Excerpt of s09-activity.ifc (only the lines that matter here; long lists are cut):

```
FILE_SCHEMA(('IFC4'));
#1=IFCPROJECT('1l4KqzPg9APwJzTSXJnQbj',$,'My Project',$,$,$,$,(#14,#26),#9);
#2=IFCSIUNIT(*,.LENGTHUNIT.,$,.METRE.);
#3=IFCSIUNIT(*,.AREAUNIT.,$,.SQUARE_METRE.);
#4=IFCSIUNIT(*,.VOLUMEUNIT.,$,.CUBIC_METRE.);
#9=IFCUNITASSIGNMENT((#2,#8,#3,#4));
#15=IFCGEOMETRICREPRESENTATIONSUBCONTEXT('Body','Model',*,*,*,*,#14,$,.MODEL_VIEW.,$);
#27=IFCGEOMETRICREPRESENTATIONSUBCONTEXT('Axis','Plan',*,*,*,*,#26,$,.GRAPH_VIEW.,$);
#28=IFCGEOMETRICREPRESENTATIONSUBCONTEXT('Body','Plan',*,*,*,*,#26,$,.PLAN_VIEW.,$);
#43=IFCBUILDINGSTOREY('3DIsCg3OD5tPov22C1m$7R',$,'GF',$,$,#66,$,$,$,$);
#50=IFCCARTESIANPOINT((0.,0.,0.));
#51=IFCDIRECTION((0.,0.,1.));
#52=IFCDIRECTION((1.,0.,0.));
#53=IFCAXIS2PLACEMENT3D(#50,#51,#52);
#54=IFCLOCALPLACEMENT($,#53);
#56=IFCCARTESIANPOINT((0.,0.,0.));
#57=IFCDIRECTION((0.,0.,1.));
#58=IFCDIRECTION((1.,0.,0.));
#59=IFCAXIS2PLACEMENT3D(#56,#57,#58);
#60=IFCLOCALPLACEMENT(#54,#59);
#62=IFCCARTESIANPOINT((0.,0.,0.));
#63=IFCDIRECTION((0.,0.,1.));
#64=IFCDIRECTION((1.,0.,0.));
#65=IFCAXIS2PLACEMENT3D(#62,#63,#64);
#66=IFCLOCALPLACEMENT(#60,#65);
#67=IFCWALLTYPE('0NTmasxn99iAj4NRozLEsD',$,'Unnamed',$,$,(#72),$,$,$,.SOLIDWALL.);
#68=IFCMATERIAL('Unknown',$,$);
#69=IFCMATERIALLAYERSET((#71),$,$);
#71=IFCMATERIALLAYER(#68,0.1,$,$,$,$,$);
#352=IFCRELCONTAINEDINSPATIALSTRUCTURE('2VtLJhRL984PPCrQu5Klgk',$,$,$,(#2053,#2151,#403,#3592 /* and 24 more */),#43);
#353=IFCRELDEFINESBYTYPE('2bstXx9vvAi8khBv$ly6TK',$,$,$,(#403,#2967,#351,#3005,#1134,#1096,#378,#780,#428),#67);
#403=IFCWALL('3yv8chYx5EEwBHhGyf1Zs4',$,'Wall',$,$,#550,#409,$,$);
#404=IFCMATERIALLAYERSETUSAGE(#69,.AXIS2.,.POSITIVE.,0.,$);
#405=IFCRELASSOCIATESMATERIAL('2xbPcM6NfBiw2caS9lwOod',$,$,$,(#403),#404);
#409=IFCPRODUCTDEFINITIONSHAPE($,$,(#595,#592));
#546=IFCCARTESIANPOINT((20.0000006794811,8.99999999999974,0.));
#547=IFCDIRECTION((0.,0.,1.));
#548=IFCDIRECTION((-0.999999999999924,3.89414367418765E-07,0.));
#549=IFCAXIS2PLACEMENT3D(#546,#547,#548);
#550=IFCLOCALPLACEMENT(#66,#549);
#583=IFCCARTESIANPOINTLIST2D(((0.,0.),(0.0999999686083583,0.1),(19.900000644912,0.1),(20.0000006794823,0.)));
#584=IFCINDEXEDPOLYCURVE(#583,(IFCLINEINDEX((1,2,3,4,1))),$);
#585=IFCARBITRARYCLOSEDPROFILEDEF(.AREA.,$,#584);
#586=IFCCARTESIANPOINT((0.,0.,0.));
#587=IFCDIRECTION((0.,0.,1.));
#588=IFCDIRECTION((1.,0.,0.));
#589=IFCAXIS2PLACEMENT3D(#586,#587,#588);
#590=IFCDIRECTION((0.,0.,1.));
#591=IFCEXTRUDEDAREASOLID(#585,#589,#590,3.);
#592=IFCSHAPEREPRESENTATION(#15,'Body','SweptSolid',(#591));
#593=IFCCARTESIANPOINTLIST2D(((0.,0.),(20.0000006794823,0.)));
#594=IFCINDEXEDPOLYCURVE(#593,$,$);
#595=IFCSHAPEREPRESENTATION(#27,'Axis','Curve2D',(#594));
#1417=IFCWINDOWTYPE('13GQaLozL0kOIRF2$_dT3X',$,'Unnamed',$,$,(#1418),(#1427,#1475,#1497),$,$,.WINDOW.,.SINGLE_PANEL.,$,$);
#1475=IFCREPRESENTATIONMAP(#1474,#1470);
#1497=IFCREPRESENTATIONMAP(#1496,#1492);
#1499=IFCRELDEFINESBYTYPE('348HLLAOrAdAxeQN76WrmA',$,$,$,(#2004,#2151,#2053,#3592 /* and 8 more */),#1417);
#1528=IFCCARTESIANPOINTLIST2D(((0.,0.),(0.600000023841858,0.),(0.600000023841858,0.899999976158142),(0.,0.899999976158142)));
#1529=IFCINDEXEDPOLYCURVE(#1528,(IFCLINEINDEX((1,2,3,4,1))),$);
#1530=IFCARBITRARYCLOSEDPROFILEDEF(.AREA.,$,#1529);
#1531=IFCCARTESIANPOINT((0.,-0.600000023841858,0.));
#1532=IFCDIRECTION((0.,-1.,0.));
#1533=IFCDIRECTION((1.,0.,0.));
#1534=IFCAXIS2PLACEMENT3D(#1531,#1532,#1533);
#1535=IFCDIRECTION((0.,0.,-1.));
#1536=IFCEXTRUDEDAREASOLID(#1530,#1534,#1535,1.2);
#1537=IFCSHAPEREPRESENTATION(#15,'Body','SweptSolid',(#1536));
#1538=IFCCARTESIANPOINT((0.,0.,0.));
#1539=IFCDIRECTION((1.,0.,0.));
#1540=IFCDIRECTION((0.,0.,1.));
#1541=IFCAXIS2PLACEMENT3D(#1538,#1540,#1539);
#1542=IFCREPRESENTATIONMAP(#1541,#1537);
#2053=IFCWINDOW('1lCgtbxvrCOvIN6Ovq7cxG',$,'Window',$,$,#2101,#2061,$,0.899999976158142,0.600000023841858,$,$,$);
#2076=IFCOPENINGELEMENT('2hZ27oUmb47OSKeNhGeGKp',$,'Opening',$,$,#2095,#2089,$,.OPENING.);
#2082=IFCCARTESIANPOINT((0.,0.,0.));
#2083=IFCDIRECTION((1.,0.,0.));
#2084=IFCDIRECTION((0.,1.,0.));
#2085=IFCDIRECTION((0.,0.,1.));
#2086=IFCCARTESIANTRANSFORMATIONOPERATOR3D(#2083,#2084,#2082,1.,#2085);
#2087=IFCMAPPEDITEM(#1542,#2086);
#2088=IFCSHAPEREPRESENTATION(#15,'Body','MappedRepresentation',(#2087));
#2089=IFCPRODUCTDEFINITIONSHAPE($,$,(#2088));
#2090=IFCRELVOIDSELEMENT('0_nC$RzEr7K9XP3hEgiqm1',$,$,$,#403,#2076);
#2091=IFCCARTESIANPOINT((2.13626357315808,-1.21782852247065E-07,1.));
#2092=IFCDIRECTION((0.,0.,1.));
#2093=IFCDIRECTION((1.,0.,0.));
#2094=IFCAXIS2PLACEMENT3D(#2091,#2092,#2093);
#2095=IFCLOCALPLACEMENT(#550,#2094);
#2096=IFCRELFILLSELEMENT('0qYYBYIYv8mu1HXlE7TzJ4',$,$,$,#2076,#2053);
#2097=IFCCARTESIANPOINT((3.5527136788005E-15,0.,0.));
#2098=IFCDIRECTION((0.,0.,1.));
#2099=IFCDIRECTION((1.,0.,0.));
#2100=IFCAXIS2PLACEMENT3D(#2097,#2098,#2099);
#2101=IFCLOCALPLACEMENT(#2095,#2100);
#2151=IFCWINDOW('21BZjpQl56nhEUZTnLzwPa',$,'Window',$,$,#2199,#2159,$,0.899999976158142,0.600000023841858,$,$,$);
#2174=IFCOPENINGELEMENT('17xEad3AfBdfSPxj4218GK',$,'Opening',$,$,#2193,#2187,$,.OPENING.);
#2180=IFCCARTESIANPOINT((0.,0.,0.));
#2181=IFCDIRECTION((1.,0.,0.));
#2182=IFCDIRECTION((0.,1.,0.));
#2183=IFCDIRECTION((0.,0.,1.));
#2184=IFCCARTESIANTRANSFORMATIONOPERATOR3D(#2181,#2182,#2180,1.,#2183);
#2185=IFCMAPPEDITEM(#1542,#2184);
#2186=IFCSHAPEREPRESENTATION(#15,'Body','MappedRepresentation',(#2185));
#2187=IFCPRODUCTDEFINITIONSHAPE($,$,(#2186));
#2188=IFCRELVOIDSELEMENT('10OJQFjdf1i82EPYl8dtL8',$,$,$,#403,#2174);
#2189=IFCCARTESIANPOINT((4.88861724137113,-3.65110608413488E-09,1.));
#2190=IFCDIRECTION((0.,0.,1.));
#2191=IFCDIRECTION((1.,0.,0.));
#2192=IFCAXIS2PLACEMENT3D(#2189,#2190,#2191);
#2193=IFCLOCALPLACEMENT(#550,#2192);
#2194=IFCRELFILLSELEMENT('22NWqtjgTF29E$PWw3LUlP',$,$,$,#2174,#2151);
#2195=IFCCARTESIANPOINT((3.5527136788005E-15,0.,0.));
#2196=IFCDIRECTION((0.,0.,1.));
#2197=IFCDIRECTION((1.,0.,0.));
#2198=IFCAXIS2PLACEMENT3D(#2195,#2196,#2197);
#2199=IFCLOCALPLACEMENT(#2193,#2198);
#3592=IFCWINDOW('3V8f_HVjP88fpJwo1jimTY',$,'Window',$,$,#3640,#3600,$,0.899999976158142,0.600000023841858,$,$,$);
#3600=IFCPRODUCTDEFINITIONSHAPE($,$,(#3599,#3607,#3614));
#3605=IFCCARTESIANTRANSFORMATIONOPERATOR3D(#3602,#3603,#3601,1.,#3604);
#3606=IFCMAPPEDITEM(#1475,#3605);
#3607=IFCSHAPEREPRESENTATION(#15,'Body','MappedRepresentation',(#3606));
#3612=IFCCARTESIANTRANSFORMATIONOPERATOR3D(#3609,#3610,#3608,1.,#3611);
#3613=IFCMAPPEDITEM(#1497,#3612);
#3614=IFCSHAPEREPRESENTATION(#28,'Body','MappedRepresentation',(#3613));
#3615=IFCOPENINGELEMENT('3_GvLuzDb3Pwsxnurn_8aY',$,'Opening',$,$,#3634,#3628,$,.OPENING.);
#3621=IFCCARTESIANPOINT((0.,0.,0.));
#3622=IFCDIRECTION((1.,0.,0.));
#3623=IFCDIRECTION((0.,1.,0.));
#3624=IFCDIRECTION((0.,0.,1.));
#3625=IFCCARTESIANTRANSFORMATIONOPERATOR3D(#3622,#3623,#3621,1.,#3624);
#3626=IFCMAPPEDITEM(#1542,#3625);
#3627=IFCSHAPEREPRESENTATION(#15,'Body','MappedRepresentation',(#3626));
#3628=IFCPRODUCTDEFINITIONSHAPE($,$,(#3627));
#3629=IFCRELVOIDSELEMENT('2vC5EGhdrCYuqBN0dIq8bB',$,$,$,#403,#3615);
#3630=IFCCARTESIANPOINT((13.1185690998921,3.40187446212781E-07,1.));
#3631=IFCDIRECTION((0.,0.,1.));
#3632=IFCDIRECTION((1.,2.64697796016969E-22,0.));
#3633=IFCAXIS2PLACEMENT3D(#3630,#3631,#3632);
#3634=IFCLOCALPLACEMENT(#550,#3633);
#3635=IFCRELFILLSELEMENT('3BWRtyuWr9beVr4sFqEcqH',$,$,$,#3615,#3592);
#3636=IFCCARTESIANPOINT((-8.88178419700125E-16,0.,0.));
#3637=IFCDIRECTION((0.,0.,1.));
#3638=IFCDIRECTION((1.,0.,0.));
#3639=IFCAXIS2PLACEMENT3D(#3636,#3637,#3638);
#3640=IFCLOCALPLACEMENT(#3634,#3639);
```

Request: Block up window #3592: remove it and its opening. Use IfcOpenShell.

```python
import ifcopenshell
import ifcopenshell.api.feature
import ifcopenshell.api.root
import ifcopenshell.geom
import ifcopenshell.util.shape

model = ifcopenshell.open("s09-activity.ifc")
settings = ifcopenshell.geom.settings()


def volume(element):
    """Net volume in cubic metres, openings subtracted."""
    shape = ifcopenshell.geom.create_shape(settings, element)
    return ifcopenshell.util.shape.get_volume(shape.geometry)


window = model.by_id(3592)
opening = window.FillsVoids[0].RelatingOpeningElement
wall = opening.VoidsElements[0].RelatingBuildingElement
before = volume(wall)

ifcopenshell.api.root.remove_product(model, product=window)
ifcopenshell.api.feature.remove_feature(model, feature=opening)

after = volume(wall)

print(f"wall volume {before:.3f} -> {after:.3f} m3")

model.write("s09-activity-out.ifc")
```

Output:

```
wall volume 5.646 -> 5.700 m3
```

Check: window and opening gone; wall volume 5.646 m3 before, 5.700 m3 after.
